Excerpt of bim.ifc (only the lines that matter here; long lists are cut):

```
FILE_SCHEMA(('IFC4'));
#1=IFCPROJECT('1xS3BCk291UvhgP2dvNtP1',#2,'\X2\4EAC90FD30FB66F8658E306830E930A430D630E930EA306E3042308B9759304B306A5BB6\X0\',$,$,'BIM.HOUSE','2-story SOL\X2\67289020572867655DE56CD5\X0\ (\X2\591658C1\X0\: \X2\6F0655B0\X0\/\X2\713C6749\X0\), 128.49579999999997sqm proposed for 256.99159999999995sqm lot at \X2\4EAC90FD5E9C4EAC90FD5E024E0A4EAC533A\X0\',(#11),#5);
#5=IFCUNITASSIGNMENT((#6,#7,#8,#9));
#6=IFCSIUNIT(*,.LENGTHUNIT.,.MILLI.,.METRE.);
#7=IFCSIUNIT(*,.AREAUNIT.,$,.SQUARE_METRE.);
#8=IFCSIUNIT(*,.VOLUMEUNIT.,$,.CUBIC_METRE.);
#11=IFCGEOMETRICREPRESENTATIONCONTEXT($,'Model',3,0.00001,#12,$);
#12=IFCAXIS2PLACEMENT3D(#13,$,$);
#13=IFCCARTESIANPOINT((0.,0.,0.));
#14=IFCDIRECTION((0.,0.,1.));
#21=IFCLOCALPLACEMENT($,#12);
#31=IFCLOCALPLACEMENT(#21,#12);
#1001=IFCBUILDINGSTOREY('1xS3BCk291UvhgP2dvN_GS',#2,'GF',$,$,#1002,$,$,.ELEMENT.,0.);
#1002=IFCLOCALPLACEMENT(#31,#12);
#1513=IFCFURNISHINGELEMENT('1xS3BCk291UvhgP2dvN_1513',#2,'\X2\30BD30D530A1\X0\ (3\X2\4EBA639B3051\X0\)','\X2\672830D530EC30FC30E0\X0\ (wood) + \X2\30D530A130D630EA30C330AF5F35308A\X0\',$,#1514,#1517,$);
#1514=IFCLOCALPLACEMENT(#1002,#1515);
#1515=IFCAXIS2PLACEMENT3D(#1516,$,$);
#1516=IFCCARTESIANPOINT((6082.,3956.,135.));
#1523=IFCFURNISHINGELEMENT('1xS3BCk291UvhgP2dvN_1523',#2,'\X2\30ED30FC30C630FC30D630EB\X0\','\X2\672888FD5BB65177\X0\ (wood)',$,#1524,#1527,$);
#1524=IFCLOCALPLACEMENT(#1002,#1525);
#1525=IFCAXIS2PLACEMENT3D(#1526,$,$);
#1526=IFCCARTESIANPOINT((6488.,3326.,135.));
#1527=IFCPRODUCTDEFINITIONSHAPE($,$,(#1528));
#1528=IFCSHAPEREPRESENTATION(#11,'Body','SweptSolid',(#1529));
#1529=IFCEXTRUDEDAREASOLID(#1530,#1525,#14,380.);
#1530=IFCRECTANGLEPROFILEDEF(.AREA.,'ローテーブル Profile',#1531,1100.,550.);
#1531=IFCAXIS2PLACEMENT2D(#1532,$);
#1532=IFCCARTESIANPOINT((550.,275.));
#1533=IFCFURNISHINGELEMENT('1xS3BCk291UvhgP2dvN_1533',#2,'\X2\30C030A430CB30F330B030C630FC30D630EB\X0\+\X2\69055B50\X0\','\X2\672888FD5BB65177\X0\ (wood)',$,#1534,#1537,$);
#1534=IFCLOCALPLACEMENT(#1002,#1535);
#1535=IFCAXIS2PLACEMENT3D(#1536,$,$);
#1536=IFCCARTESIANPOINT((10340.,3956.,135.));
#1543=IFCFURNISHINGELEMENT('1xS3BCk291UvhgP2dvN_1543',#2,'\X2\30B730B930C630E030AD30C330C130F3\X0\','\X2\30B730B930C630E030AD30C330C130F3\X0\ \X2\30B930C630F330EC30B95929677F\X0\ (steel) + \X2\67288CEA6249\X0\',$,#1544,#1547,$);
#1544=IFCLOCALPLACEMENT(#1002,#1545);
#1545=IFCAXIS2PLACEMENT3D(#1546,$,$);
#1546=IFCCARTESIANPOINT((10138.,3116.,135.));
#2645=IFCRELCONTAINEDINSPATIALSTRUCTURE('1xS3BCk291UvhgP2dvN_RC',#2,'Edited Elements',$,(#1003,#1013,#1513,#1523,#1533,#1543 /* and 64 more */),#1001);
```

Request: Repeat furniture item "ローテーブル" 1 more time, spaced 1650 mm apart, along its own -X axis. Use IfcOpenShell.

```python
import ifcopenshell
import ifcopenshell.api.geometry
import ifcopenshell.api.root
import ifcopenshell.util.element
import ifcopenshell.util.placement
import ifcopenshell.util.unit

model = ifcopenshell.open("bim.ifc")
unit_scale = ifcopenshell.util.unit.calculate_unit_scale(model)


def reuse_history(source, copy):
    """copy_class also copies each property set's owner history, people and application; keep the originals."""
    for rel in copy.IsDefinedBy:
        if rel.is_a("IfcRelDefinesByProperties") and (history := rel.RelatingPropertyDefinition.OwnerHistory):
            rel.RelatingPropertyDefinition.OwnerHistory = source.OwnerHistory
            ifcopenshell.util.element.remove_deep2(model, history)


source = model.by_guid("1xS3BCk291UvhgP2dvN_1523")
base = ifcopenshell.util.placement.get_local_placement(source.ObjectPlacement)
step = -base[:3, 0] * 1.65 / unit_scale

for i in range(1, 2):
    copy = ifcopenshell.api.root.copy_class(model, product=source)
    copy.Representation = ifcopenshell.util.element.copy_deep(
        model, source.Representation, exclude=["IfcGeometricRepresentationContext", "IfcRepresentationMap"]
    )
    reuse_history(source, copy)
    matrix = base.copy()
    matrix[:3, 3] += i * step
    print("added at", matrix[:3, 3].round(3) + 0.0)
    ifcopenshell.api.geometry.edit_object_placement(model, product=copy, matrix=matrix, is_si=False)

model.write("bim_edited.ifc")
```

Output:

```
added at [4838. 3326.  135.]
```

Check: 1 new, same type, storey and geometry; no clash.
